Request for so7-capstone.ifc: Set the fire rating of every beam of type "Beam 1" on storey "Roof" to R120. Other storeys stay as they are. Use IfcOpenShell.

First a look at what the model holds.

```python
import ifcopenshell
import ifcopenshell.util.element

model = ifcopenshell.open("so7-capstone.ifc")
print(model.schema)
storey = next(s for s in model.by_type("IfcBuildingStorey") if s.Name == "Roof")
beams = [e for e in ifcopenshell.util.element.get_decomposition(storey) if e.is_a("IfcBeam")]
seen = {}
for e in beams:
    element_type = ifcopenshell.util.element.get_type(e)
    key = (element_type.Name if element_type != e and element_type else None, ifcopenshell.util.element.get_pset(e, "Pset_BeamCommon", "FireRating"))
    seen[key] = seen.get(key, 0) + 1
for (name, value), count in sorted(seen.items(), key=str):
    print(count, "x", name, "|", value)
```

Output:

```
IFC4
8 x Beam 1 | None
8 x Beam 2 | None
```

```python
import ifcopenshell
import ifcopenshell.api.pset
import ifcopenshell.util.element

model = ifcopenshell.open("so7-capstone.ifc")

storey = next(s for s in model.by_type("IfcBuildingStorey") if s.Name == "Roof")
beams = [e for e in ifcopenshell.util.element.get_decomposition(storey) if e.is_a("IfcBeam")]

count = 0
for e in beams:
    element_type = ifcopenshell.util.element.get_type(e)
    if element_type in (None, e) or element_type.Name != "Beam 1":
        continue
    # add_pset returns the element's existing set when there is one.
    pset = ifcopenshell.api.pset.add_pset(model, product=e, name="Pset_BeamCommon")
    ifcopenshell.api.pset.edit_pset(model, pset=pset, properties={"FireRating": "R120"})
    count += 1

print(count, "beams updated")

model.write("so7-capstone_updated.ifc")
```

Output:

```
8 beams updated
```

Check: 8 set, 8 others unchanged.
